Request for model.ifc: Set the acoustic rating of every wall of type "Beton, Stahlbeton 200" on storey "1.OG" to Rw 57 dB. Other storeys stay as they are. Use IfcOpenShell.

First a look at what the model holds.

```python
import ifcopenshell
import ifcopenshell.util.element

model = ifcopenshell.open("model.ifc")
print(model.schema)
storey = next(s for s in model.by_type("IfcBuildingStorey") if s.Name == "1.OG")
walls = [e for e in ifcopenshell.util.element.get_decomposition(storey) if e.is_a("IfcWall")]
seen = {}
for e in walls:
    element_type = ifcopenshell.util.element.get_type(e)
    key = (element_type.Name if element_type != e and element_type else None, ifcopenshell.util.element.get_pset(e, "Pset_WallCommon", "AcousticRating"))
    seen[key] = seen.get(key, 0) + 1
for (name, value), count in sorted(seen.items(), key=str):
    print(count, "x", name, "|", value)
```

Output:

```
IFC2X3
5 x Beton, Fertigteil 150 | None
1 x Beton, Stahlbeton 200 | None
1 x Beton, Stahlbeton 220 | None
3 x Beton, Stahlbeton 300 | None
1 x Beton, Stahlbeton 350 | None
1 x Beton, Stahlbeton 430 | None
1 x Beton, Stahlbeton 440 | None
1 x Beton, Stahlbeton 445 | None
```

```python
import ifcopenshell
import ifcopenshell.api.pset
import ifcopenshell.util.element

model = ifcopenshell.open("model.ifc")

storey = next(s for s in model.by_type("IfcBuildingStorey") if s.Name == "1.OG")
walls = [e for e in ifcopenshell.util.element.get_decomposition(storey) if e.is_a("IfcWall")]

count = 0
for e in walls:
    element_type = ifcopenshell.util.element.get_type(e)
    if element_type in (None, e) or element_type.Name != "Beton, Stahlbeton 200":
        continue
    # add_pset returns the element's existing set when there is one.
    pset = ifcopenshell.api.pset.add_pset(model, product=e, name="Pset_WallCommon")
    ifcopenshell.api.pset.edit_pset(model, pset=pset, properties={"AcousticRating": "Rw 57 dB"})
    count += 1

print(count, "walls updated")

model.write("model_rev.ifc")
```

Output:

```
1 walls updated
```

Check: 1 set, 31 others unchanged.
